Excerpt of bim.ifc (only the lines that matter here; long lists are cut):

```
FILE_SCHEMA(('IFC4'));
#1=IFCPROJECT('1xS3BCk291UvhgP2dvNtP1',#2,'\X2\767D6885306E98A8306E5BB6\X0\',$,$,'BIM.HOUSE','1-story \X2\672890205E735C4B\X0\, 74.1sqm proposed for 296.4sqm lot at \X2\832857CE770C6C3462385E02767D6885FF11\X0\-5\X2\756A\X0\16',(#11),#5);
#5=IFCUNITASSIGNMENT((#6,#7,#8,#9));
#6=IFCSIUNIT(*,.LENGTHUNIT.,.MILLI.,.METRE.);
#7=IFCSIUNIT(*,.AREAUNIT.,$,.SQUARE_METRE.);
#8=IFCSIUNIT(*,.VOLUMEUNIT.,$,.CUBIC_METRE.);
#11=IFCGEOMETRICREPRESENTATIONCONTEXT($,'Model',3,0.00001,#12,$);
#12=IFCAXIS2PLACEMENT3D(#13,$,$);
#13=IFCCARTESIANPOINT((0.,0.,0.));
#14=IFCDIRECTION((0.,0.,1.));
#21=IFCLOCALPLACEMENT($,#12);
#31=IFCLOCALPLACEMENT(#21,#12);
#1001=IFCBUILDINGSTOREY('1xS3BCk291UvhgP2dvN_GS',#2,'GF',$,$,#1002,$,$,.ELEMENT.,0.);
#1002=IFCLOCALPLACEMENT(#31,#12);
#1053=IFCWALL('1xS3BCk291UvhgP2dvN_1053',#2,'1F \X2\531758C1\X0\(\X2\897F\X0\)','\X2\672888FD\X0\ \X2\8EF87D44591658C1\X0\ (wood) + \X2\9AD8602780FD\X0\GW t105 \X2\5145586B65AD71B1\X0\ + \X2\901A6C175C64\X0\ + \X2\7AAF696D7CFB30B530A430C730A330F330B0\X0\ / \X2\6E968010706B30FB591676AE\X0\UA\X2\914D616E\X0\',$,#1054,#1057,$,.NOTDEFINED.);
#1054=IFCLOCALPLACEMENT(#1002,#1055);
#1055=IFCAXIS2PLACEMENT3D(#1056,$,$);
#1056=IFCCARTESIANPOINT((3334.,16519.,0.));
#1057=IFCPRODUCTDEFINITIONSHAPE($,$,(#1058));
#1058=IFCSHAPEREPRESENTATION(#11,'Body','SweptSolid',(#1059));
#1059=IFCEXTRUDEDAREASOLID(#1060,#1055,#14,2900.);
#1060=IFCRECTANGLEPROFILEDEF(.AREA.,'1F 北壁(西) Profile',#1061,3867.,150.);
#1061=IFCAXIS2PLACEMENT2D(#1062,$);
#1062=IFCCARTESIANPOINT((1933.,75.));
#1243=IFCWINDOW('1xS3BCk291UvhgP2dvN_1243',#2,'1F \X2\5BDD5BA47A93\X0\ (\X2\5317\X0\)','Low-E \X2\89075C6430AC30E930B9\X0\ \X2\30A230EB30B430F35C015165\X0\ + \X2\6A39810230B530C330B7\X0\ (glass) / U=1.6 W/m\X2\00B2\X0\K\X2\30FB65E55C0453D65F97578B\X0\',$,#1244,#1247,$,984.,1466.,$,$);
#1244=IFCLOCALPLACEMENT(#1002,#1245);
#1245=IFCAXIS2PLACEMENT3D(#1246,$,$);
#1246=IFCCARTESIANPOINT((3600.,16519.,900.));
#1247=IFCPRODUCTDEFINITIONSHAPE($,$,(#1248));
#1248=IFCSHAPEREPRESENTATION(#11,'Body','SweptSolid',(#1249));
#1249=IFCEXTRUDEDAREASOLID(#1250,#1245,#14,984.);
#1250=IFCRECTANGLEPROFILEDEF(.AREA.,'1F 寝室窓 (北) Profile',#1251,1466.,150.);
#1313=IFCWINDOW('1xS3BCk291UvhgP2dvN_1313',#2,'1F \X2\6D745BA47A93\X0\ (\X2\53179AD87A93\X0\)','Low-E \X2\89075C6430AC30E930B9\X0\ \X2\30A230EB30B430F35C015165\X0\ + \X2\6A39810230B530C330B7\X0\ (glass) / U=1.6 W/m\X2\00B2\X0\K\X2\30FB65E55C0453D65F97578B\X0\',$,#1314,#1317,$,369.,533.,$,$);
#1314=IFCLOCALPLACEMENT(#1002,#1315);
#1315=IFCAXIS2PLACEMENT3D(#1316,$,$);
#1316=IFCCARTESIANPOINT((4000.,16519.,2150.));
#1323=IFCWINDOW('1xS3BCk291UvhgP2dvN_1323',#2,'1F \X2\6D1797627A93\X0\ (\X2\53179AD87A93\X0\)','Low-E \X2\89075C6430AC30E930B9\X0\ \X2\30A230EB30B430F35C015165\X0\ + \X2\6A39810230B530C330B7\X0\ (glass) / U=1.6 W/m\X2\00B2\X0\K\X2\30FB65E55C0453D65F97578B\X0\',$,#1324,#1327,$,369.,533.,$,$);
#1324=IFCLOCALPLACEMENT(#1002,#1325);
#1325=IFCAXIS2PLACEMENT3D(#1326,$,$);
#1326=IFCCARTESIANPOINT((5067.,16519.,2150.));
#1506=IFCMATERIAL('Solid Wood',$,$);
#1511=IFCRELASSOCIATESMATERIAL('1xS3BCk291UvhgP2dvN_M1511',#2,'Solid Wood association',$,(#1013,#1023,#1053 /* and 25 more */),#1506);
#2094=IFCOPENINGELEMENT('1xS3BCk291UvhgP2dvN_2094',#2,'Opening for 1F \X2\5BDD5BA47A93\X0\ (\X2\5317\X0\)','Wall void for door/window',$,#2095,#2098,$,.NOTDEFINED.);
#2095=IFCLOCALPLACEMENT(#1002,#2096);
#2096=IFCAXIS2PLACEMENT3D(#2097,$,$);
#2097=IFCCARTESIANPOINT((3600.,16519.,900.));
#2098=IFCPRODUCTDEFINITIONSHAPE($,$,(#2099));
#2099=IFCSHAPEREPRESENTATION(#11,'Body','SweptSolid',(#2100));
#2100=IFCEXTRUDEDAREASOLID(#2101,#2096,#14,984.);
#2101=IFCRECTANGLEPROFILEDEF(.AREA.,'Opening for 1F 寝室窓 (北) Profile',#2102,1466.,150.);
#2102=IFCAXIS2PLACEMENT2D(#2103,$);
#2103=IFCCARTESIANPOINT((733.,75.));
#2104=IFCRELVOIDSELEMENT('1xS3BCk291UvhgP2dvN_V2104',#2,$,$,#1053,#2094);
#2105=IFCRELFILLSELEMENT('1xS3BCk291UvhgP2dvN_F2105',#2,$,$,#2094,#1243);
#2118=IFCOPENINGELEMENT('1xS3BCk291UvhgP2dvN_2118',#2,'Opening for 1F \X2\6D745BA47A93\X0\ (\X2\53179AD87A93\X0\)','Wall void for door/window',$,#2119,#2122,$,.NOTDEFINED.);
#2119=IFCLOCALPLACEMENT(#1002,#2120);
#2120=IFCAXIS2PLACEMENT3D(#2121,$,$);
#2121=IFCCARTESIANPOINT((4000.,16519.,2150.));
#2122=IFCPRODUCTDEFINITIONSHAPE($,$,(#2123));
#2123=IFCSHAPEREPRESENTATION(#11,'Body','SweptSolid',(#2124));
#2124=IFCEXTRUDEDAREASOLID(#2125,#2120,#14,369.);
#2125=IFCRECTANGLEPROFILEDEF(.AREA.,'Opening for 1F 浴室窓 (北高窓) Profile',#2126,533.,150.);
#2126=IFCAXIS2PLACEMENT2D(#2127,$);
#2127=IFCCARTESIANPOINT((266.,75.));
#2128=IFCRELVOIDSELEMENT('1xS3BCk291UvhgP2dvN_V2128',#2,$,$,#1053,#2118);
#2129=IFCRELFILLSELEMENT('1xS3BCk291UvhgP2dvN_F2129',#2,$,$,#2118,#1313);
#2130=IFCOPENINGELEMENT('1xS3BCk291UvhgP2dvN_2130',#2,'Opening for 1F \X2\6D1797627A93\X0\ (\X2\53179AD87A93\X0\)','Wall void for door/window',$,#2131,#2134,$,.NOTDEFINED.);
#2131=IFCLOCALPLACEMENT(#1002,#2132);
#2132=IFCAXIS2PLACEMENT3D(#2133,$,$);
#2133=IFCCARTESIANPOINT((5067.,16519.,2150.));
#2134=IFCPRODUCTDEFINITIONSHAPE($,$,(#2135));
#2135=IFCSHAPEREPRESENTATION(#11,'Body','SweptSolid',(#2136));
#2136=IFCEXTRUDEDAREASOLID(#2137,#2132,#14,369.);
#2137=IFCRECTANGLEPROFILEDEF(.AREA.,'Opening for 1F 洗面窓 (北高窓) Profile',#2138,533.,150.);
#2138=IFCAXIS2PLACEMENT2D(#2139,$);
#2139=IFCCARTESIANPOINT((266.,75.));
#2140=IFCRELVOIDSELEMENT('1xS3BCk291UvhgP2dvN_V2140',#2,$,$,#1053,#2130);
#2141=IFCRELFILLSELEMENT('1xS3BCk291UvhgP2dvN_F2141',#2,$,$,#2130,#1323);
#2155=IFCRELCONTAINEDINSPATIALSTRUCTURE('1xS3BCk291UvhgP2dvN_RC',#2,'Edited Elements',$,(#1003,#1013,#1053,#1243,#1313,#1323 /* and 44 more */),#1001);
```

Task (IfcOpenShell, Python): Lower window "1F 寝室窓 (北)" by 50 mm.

```python
import numpy as np
import ifcopenshell
import ifcopenshell.api.geometry
import ifcopenshell.util.placement
import ifcopenshell.util.unit

model = ifcopenshell.open("bim.ifc")
unit_scale = ifcopenshell.util.unit.calculate_unit_scale(model)

window = model.by_guid("1xS3BCk291UvhgP2dvN_1243")
opening = window.FillsVoids[0].RelatingOpeningElement
dz = -50.0

shift = np.array([0.0, 0.0, dz])
# The window is not placed relative to its opening, so move both.
for product in (opening, window):
    matrix = ifcopenshell.util.placement.get_local_placement(product.ObjectPlacement)
    matrix[:3, 3] += shift
    ifcopenshell.api.geometry.edit_object_placement(model, product=product, matrix=matrix, is_si=False)

print(f"moved by {dz * unit_scale:+.3f} m")

model.write("bim_rev.ifc")
```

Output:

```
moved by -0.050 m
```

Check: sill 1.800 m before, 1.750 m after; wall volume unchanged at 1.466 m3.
